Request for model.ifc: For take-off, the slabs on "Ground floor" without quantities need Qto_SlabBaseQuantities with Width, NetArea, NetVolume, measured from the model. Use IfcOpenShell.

First a look at what the model holds.

```python
import ifcopenshell
import ifcopenshell.util.element
import ifcopenshell.util.unit

model = ifcopenshell.open("model.ifc")
print(model.schema)
for unit_type in ("LENGTHUNIT", "AREAUNIT", "VOLUMEUNIT"):
    print(unit_type, ifcopenshell.util.unit.calculate_unit_scale(model, unit_type))
storey = next(s for s in model.by_type("IfcBuildingStorey") if s.Name == "Ground floor")
slabs = [e for e in ifcopenshell.util.element.get_decomposition(storey) if e.is_a("IfcSlab")]
for e in sorted(slabs, key=lambda e: e.id()):
    print(e.id(), e.is_a(), e.Name, list(ifcopenshell.util.element.get_psets(e, qtos_only=True)), sep=" | ")
```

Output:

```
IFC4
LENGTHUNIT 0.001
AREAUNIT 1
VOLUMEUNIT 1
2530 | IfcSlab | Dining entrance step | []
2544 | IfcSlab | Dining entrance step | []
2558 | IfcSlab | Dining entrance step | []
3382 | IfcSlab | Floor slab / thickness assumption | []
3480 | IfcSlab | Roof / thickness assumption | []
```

```python
import ifcopenshell
import ifcopenshell.api.pset
import ifcopenshell.geom
import ifcopenshell.util.element
import ifcopenshell.util.shape
import ifcopenshell.util.unit

model = ifcopenshell.open("model.ifc")
unit_scale = ifcopenshell.util.unit.calculate_unit_scale(model)
area_scale = ifcopenshell.util.unit.calculate_unit_scale(model, "AREAUNIT")
volume_scale = ifcopenshell.util.unit.calculate_unit_scale(model, "VOLUMEUNIT")
settings = ifcopenshell.geom.settings()

storey = next(s for s in model.by_type("IfcBuildingStorey") if s.Name == "Ground floor")
slabs = [e for e in ifcopenshell.util.element.get_decomposition(storey) if e.is_a("IfcSlab")]

for e in sorted(slabs, key=lambda e: e.id()):
    if ifcopenshell.util.element.get_psets(e, qtos_only=True, should_inherit=False):
        continue
    # Geometry comes back in metres, in the element's own axes.
    shape = ifcopenshell.geom.create_shape(settings, e)
    values = {
        "Width": ifcopenshell.util.shape.get_z(shape.geometry) / unit_scale,
        "NetArea": ifcopenshell.util.shape.get_footprint_area(shape.geometry) / area_scale,
        "NetVolume": ifcopenshell.util.shape.get_volume(shape.geometry) / volume_scale,
    }
    qto = ifcopenshell.api.pset.add_qto(model, product=e, name="Qto_SlabBaseQuantities")
    ifcopenshell.api.pset.edit_qto(model, qto=qto, properties=values)
    print(e.id(), {k: round(v, 3) for k, v in values.items()})

model.write("model-out.ifc")
```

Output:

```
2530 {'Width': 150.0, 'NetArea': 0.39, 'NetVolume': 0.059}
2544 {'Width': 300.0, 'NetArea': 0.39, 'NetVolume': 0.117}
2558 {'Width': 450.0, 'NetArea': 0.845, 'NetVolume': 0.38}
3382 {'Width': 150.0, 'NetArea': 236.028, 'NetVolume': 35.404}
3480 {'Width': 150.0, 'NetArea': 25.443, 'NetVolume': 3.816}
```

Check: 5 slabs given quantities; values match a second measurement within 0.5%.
